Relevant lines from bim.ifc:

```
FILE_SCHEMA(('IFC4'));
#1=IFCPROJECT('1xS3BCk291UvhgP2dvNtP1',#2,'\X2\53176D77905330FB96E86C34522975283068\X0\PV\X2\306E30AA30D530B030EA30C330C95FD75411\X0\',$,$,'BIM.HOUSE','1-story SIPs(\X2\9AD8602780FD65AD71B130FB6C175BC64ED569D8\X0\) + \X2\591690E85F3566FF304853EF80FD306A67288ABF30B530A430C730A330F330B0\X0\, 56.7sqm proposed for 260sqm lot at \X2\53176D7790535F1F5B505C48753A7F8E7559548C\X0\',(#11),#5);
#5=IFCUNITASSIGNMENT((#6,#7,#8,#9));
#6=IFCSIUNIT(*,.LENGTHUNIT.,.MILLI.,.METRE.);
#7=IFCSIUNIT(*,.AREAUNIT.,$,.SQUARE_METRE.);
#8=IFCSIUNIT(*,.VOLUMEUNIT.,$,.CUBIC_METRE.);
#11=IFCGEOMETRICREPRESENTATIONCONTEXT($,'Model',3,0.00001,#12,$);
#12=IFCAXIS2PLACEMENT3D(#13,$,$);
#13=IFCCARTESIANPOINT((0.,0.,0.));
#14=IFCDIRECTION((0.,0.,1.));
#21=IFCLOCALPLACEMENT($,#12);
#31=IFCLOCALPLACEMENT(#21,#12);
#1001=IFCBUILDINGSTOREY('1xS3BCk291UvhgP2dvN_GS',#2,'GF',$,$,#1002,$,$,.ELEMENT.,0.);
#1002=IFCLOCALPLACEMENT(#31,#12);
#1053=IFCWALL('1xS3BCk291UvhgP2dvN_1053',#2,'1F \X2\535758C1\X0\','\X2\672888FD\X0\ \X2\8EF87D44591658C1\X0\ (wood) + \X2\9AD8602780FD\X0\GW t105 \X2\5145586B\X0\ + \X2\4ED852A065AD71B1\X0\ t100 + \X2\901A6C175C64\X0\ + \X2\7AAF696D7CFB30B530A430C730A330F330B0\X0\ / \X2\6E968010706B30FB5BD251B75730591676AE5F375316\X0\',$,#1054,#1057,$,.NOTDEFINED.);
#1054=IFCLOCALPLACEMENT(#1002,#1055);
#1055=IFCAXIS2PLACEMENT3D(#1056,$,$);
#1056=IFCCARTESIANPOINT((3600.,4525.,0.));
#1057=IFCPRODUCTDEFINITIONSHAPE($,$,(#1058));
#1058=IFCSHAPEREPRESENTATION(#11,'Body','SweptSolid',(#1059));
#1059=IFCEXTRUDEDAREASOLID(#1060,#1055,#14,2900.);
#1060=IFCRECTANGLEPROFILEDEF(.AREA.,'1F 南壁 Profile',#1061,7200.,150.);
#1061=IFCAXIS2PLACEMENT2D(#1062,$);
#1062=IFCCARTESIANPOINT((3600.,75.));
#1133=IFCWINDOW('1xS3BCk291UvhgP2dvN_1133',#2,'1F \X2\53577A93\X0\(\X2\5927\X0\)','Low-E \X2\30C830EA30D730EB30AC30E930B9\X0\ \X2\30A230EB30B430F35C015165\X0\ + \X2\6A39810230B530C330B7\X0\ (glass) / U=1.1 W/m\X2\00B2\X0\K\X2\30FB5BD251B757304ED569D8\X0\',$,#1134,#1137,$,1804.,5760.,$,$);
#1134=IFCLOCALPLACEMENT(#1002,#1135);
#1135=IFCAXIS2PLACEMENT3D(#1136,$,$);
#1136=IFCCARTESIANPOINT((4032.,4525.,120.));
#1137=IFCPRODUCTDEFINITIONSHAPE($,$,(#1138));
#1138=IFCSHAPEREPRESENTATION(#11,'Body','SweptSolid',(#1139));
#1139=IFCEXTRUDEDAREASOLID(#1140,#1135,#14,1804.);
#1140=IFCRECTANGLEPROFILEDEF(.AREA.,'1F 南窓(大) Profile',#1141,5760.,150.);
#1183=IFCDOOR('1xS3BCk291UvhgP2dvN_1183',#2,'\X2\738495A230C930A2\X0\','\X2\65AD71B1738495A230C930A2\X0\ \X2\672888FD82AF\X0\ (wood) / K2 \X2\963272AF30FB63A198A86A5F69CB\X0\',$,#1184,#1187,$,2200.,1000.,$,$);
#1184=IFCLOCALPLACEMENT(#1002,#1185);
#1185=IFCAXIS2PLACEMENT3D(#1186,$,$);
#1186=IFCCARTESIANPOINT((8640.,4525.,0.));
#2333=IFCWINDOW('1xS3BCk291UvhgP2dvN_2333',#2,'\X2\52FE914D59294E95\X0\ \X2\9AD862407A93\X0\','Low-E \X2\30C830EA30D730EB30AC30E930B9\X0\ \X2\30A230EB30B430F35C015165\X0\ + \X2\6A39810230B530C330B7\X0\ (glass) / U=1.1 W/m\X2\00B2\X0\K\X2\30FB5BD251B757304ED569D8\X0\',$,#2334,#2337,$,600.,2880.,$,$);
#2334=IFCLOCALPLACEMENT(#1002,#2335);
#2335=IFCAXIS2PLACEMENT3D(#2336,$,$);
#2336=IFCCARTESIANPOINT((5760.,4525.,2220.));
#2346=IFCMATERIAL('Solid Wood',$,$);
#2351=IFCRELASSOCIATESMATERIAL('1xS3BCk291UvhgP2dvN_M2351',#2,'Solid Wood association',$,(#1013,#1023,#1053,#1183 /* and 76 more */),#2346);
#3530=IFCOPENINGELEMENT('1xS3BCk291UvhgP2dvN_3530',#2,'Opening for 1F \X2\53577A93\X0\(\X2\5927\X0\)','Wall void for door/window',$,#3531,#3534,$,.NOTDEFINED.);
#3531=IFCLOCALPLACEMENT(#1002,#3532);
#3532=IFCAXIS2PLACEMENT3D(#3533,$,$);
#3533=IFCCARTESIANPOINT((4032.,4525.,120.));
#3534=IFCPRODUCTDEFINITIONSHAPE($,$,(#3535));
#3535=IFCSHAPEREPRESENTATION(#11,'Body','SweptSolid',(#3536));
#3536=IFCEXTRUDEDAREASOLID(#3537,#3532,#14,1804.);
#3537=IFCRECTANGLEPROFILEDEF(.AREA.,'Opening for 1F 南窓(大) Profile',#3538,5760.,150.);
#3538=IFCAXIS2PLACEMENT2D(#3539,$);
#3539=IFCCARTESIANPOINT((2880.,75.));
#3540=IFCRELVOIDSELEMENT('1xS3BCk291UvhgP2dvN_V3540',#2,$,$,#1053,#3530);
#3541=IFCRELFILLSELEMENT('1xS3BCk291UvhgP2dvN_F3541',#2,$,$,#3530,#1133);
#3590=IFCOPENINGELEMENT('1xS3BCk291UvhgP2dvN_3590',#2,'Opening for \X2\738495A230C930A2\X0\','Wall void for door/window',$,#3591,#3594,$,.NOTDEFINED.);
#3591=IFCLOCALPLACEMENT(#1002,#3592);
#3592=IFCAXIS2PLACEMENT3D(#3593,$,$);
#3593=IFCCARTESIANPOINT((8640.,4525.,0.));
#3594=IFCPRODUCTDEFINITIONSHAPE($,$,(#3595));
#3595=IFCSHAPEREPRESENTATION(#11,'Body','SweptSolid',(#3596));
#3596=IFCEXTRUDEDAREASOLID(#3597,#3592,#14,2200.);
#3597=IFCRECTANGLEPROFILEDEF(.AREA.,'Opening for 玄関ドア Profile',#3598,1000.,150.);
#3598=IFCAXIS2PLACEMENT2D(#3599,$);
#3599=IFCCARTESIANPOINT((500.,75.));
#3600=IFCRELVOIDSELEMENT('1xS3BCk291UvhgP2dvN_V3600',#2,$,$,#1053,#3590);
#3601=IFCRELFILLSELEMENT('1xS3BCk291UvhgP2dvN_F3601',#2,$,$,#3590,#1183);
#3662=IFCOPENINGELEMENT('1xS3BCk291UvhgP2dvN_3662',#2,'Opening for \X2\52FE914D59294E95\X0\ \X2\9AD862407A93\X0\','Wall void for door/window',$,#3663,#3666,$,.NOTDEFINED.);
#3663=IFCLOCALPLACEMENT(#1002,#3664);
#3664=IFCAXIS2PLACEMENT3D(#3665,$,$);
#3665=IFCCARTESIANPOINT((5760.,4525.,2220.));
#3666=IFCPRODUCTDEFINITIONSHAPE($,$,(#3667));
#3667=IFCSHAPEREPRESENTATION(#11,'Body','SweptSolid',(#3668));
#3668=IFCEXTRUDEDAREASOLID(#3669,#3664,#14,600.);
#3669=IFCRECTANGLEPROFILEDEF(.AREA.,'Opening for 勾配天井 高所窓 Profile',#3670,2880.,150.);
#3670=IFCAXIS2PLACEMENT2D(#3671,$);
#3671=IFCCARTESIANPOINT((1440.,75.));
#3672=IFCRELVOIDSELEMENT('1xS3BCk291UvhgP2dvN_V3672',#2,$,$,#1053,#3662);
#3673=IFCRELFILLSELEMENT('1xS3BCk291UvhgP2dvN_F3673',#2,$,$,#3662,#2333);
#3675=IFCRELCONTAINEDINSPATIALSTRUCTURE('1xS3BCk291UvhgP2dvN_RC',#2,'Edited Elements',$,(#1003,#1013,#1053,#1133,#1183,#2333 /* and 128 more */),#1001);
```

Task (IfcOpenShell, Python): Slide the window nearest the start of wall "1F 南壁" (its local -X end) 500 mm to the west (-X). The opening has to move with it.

```python
import ifcopenshell
import ifcopenshell.api.geometry
import ifcopenshell.util.placement

model = ifcopenshell.open("bim.ifc")

window = model.by_guid("1xS3BCk291UvhgP2dvN_1133")
opening = window.FillsVoids[0].RelatingOpeningElement
wall = opening.VoidsElements[0].RelatingBuildingElement

wall_matrix = ifcopenshell.util.placement.get_local_placement(wall.ObjectPlacement)
shift = wall_matrix[:3, 0] * -500.0
before = ifcopenshell.util.placement.get_local_placement(window.ObjectPlacement)[:3, 3].copy()

# The window is not placed relative to its opening, so move both.
for product in (opening, window):
    matrix = ifcopenshell.util.placement.get_local_placement(product.ObjectPlacement)
    matrix[:3, 3] += shift
    ifcopenshell.api.geometry.edit_object_placement(model, product=product, matrix=matrix, is_si=False)

after = ifcopenshell.util.placement.get_local_placement(window.ObjectPlacement)[:3, 3]
print("window moved by", (after - before).round(3) + 0.0)

model.write("bim-out.ifc")
```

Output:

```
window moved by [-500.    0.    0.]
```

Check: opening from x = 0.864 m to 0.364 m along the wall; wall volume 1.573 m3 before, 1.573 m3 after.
